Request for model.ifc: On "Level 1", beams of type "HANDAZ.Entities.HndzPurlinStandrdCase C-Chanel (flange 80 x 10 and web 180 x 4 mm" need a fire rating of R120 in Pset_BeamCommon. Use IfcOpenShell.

First a look at what the model holds.

```python
import ifcopenshell
import ifcopenshell.util.element

model = ifcopenshell.open("model.ifc")
print(model.schema)
storey = next(s for s in model.by_type("IfcBuildingStorey") if s.Name == "Level 1")
beams = [e for e in ifcopenshell.util.element.get_decomposition(storey) if e.is_a("IfcBeam")]
seen = {}
for e in beams:
    element_type = ifcopenshell.util.element.get_type(e)
    key = (element_type.Name if element_type != e and element_type else None, ifcopenshell.util.element.get_pset(e, "Pset_BeamCommon", "FireRating"))
    seen[key] = seen.get(key, 0) + 1
for (name, value), count in sorted(seen.items(), key=str):
    print(count, "x", name, "|", value)
```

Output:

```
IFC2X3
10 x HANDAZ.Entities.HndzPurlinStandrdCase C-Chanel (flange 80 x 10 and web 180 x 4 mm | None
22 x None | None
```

```python
import ifcopenshell
import ifcopenshell.api.pset
import ifcopenshell.util.element

model = ifcopenshell.open("model.ifc")

storey = next(s for s in model.by_type("IfcBuildingStorey") if s.Name == "Level 1")
beams = [e for e in ifcopenshell.util.element.get_decomposition(storey) if e.is_a("IfcBeam")]

count = 0
for e in beams:
    element_type = ifcopenshell.util.element.get_type(e)
    if element_type in (None, e) or element_type.Name != "HANDAZ.Entities.HndzPurlinStandrdCase C-Chanel (flange 80 x 10 and web 180 x 4 mm":
        continue
    # add_pset returns the element's existing set when there is one.
    pset = ifcopenshell.api.pset.add_pset(model, product=e, name="Pset_BeamCommon")
    ifcopenshell.api.pset.edit_pset(model, pset=pset, properties={"FireRating": "R120"})
    count += 1

print(count, "beams updated")

model.write("model_edited.ifc")
```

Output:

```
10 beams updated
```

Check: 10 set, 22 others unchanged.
